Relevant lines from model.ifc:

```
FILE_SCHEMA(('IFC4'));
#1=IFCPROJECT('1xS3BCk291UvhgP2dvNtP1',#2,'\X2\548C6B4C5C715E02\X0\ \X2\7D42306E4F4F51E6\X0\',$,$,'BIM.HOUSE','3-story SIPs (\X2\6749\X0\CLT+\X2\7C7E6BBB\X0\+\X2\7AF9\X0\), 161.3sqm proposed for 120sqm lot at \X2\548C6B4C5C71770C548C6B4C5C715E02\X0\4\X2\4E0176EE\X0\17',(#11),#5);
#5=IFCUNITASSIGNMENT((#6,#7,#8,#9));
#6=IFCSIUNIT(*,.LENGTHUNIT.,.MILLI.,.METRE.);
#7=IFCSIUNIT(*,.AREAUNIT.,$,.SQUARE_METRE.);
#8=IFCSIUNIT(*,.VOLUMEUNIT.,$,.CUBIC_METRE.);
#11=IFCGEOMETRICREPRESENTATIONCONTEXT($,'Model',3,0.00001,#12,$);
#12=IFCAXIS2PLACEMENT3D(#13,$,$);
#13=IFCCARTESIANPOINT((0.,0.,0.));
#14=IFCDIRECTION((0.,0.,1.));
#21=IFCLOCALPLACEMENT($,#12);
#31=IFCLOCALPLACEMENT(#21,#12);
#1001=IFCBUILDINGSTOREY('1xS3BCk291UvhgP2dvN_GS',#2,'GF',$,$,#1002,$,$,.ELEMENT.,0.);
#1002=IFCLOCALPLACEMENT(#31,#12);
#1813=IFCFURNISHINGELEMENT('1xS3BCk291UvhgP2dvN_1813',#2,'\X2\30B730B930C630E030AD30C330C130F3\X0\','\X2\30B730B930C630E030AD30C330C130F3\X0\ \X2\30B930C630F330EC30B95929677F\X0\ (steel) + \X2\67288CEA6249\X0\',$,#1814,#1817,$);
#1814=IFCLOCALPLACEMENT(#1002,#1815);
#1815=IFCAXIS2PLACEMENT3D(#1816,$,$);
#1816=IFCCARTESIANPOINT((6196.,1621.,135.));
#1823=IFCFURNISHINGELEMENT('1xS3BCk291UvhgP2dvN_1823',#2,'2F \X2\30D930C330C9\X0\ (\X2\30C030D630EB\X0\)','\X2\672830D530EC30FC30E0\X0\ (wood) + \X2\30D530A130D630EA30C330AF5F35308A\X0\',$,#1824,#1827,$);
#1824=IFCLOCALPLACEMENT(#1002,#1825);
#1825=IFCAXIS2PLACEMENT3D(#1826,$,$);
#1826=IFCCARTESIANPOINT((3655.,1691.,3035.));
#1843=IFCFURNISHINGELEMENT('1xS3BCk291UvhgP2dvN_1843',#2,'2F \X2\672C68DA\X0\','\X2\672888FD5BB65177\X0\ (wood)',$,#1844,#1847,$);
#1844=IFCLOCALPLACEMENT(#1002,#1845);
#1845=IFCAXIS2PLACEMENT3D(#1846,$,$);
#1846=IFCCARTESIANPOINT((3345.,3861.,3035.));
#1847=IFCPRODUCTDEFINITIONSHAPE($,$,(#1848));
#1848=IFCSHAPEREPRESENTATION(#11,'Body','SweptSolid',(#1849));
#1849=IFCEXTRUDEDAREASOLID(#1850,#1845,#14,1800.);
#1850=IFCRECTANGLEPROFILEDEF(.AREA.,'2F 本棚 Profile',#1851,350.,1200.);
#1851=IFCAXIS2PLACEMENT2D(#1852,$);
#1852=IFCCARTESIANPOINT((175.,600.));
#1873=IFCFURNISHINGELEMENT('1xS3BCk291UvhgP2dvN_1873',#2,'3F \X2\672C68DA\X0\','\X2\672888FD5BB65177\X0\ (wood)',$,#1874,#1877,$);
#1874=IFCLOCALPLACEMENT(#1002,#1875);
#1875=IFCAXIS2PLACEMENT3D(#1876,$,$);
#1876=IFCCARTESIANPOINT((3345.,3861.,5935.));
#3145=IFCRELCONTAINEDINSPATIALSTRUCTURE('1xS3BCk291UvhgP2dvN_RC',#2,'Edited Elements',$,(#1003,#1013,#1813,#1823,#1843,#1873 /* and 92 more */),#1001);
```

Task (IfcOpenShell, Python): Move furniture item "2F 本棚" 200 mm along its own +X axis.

```python
import ifcopenshell
import ifcopenshell.api.geometry
import ifcopenshell.util.placement

model = ifcopenshell.open("model.ifc")

item = model.by_guid("1xS3BCk291UvhgP2dvN_1843")
matrix = ifcopenshell.util.placement.get_local_placement(item.ObjectPlacement)
matrix[:3, 3] += matrix[:3, 0] * 200.0
ifcopenshell.api.geometry.edit_object_placement(model, product=item, matrix=matrix, is_si=False)

print(ifcopenshell.util.placement.get_local_placement(item.ObjectPlacement).round(3) + 0.0)

model.write("model_updated.ifc")
```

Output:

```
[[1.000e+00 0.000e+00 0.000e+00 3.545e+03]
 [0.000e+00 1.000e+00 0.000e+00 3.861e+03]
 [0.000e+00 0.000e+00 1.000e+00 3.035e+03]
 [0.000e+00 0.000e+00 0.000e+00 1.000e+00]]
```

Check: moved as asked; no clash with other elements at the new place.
